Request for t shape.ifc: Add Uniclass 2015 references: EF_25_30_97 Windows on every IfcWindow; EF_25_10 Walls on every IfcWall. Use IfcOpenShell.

First a look at what the model holds.

```python
import ifcopenshell

model = ifcopenshell.open("t shape.ifc")
print(model.schema)
print("classifications:", [c.Name for c in model.by_type("IfcClassification")])
for ifc_class in ("IfcDoor", "IfcRoof", "IfcStair", "IfcWall", "IfcWindow"):
    print(ifc_class, len(model.by_type(ifc_class)))
```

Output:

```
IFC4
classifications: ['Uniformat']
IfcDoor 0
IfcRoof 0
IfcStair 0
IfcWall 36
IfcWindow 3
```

```python
import ifcopenshell
import ifcopenshell.api.classification

model = ifcopenshell.open("t shape.ifc")

system = ifcopenshell.api.classification.add_classification(model, classification="Uniclass 2015")

codes = {
    "IfcWindow": ("EF_25_30_97", "Windows"),
    "IfcWall": ("EF_25_10", "Walls"),
}
for ifc_class, (code, name) in codes.items():
    products = model.by_type(ifc_class)
    ifcopenshell.api.classification.add_reference(
        model, products=products, classification=system, identification=code, name=name
    )
    print(code, len(products))

model.write("t shape-out.ifc")
```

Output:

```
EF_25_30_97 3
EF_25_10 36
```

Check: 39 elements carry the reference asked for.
